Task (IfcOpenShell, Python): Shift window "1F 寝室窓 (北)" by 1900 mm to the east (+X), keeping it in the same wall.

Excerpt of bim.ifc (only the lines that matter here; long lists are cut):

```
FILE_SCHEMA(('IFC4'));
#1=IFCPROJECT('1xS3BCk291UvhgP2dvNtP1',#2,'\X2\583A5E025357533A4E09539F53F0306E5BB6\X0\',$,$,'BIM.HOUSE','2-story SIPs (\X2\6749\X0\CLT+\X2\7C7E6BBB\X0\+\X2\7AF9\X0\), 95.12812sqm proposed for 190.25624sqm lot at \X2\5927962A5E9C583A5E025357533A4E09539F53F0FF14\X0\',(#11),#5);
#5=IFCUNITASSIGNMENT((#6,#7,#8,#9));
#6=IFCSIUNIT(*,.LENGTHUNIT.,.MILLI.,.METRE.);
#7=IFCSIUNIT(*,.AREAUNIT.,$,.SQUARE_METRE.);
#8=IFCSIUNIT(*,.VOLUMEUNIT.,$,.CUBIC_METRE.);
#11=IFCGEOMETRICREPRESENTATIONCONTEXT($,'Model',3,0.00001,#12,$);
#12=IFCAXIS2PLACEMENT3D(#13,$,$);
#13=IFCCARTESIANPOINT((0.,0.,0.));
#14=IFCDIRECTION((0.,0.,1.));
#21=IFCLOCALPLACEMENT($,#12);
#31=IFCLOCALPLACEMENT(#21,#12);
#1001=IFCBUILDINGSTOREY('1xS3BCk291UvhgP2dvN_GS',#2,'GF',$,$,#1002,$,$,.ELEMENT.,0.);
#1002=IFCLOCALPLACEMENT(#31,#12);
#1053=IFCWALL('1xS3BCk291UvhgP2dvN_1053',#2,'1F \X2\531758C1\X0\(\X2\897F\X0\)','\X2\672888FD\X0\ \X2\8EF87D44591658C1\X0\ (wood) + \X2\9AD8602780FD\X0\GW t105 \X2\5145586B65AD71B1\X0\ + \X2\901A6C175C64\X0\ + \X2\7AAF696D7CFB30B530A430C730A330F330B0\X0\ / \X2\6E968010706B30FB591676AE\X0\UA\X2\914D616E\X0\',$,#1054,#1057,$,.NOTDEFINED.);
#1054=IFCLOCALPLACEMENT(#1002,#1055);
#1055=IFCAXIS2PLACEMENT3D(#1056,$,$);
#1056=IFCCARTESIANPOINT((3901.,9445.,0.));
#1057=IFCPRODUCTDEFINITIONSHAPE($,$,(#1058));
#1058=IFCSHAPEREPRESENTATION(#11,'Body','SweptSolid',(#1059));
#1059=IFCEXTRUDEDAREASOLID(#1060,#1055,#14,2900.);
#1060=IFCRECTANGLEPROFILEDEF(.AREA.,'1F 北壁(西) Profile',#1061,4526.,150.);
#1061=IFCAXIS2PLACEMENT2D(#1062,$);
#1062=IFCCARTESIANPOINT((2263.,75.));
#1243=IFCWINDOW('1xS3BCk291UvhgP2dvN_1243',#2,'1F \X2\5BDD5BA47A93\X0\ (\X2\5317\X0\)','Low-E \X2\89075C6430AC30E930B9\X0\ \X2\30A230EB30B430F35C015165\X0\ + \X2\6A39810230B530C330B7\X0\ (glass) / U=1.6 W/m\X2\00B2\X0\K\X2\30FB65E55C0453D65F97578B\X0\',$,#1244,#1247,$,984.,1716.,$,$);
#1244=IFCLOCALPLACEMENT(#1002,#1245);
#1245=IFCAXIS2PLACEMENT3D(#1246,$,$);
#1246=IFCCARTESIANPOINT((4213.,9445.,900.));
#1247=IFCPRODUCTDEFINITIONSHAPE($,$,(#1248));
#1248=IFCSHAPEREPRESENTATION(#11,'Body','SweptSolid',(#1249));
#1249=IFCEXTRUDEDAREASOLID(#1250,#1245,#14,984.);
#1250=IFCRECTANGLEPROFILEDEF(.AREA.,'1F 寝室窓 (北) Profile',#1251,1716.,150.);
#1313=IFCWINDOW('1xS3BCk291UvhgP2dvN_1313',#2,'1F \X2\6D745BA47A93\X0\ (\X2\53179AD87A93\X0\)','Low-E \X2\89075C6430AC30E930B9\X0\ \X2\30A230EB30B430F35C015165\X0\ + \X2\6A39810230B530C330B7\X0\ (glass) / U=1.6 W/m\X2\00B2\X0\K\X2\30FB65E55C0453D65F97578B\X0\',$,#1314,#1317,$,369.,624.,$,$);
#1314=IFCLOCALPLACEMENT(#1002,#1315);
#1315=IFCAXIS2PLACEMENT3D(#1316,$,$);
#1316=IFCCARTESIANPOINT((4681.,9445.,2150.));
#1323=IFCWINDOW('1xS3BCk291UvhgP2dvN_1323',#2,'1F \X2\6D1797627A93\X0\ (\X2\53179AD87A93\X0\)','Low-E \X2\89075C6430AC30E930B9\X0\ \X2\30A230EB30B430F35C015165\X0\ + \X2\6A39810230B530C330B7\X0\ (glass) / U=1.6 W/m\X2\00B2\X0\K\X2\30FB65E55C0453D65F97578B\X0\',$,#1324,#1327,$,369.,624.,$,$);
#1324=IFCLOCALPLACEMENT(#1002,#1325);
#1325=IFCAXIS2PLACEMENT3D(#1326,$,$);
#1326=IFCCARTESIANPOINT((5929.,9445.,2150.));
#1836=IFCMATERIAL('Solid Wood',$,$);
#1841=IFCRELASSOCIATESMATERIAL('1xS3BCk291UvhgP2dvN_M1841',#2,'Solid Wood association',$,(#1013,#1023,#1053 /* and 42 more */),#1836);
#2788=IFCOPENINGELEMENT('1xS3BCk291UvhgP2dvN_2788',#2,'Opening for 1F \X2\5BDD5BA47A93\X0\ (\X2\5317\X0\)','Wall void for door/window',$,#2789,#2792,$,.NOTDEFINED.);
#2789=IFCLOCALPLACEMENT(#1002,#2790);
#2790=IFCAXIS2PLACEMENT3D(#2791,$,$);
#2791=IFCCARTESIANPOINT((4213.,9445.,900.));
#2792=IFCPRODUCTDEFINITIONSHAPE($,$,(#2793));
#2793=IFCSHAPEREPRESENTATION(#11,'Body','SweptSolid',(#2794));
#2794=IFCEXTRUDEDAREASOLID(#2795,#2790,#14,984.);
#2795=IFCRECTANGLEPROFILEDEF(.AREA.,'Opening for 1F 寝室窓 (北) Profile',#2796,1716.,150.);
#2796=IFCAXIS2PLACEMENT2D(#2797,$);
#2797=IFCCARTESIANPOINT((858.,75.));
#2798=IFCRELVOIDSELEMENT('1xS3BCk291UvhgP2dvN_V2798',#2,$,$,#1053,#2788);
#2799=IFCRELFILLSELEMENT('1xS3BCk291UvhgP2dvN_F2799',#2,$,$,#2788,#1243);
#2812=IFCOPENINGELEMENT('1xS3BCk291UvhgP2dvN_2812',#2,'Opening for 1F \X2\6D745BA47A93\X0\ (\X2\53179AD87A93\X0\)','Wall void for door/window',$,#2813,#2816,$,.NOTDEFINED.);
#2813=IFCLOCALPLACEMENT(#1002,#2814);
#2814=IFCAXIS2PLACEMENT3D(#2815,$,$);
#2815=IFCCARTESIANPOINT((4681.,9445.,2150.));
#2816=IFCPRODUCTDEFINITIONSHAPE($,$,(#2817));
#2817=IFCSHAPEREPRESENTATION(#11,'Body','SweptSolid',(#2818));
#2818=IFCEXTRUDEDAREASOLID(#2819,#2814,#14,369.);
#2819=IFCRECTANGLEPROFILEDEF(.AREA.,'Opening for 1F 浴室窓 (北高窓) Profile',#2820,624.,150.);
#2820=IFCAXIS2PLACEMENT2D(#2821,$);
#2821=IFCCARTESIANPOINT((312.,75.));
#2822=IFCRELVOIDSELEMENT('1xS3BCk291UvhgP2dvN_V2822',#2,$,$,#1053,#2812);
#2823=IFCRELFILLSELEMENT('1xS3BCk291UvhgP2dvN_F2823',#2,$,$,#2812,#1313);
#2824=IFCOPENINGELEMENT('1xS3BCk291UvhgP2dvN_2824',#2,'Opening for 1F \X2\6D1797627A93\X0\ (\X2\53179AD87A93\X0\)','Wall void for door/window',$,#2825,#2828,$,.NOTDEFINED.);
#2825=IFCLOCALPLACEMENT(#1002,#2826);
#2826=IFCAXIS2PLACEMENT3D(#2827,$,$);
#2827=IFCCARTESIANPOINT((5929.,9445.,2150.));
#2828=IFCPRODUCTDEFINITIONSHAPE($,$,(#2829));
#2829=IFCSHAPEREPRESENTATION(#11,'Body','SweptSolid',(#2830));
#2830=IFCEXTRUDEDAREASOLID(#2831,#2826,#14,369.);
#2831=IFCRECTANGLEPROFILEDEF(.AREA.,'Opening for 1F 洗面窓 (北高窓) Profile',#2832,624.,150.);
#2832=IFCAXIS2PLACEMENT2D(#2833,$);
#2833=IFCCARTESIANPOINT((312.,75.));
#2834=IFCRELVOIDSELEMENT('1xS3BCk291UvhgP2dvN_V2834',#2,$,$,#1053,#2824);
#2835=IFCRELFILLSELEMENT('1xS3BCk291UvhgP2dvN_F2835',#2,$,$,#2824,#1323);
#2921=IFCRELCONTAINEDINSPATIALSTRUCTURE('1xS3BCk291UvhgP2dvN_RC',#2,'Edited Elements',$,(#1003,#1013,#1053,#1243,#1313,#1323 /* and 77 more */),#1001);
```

```python
import ifcopenshell
import ifcopenshell.api.geometry
import ifcopenshell.util.placement
import ifcopenshell.util.unit

model = ifcopenshell.open("bim.ifc")
unit_scale = ifcopenshell.util.unit.calculate_unit_scale(model)

window = model.by_guid("1xS3BCk291UvhgP2dvN_1243")
opening = window.FillsVoids[0].RelatingOpeningElement
wall = opening.VoidsElements[0].RelatingBuildingElement

wall_matrix = ifcopenshell.util.placement.get_local_placement(wall.ObjectPlacement)
shift = wall_matrix[:3, 0] * 1.9 / unit_scale
before = ifcopenshell.util.placement.get_local_placement(window.ObjectPlacement)[:3, 3].copy()

# The window is not placed relative to its opening, so move both.
for product in (opening, window):
    matrix = ifcopenshell.util.placement.get_local_placement(product.ObjectPlacement)
    matrix[:3, 3] += shift
    ifcopenshell.api.geometry.edit_object_placement(model, product=product, matrix=matrix, is_si=False)

after = ifcopenshell.util.placement.get_local_placement(window.ObjectPlacement)[:3, 3]
print("window moved by", (after - before).round(3) + 0.0)

model.write("bim-out.ifc")
```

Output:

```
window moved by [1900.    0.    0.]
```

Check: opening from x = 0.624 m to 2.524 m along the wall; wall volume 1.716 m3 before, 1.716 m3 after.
